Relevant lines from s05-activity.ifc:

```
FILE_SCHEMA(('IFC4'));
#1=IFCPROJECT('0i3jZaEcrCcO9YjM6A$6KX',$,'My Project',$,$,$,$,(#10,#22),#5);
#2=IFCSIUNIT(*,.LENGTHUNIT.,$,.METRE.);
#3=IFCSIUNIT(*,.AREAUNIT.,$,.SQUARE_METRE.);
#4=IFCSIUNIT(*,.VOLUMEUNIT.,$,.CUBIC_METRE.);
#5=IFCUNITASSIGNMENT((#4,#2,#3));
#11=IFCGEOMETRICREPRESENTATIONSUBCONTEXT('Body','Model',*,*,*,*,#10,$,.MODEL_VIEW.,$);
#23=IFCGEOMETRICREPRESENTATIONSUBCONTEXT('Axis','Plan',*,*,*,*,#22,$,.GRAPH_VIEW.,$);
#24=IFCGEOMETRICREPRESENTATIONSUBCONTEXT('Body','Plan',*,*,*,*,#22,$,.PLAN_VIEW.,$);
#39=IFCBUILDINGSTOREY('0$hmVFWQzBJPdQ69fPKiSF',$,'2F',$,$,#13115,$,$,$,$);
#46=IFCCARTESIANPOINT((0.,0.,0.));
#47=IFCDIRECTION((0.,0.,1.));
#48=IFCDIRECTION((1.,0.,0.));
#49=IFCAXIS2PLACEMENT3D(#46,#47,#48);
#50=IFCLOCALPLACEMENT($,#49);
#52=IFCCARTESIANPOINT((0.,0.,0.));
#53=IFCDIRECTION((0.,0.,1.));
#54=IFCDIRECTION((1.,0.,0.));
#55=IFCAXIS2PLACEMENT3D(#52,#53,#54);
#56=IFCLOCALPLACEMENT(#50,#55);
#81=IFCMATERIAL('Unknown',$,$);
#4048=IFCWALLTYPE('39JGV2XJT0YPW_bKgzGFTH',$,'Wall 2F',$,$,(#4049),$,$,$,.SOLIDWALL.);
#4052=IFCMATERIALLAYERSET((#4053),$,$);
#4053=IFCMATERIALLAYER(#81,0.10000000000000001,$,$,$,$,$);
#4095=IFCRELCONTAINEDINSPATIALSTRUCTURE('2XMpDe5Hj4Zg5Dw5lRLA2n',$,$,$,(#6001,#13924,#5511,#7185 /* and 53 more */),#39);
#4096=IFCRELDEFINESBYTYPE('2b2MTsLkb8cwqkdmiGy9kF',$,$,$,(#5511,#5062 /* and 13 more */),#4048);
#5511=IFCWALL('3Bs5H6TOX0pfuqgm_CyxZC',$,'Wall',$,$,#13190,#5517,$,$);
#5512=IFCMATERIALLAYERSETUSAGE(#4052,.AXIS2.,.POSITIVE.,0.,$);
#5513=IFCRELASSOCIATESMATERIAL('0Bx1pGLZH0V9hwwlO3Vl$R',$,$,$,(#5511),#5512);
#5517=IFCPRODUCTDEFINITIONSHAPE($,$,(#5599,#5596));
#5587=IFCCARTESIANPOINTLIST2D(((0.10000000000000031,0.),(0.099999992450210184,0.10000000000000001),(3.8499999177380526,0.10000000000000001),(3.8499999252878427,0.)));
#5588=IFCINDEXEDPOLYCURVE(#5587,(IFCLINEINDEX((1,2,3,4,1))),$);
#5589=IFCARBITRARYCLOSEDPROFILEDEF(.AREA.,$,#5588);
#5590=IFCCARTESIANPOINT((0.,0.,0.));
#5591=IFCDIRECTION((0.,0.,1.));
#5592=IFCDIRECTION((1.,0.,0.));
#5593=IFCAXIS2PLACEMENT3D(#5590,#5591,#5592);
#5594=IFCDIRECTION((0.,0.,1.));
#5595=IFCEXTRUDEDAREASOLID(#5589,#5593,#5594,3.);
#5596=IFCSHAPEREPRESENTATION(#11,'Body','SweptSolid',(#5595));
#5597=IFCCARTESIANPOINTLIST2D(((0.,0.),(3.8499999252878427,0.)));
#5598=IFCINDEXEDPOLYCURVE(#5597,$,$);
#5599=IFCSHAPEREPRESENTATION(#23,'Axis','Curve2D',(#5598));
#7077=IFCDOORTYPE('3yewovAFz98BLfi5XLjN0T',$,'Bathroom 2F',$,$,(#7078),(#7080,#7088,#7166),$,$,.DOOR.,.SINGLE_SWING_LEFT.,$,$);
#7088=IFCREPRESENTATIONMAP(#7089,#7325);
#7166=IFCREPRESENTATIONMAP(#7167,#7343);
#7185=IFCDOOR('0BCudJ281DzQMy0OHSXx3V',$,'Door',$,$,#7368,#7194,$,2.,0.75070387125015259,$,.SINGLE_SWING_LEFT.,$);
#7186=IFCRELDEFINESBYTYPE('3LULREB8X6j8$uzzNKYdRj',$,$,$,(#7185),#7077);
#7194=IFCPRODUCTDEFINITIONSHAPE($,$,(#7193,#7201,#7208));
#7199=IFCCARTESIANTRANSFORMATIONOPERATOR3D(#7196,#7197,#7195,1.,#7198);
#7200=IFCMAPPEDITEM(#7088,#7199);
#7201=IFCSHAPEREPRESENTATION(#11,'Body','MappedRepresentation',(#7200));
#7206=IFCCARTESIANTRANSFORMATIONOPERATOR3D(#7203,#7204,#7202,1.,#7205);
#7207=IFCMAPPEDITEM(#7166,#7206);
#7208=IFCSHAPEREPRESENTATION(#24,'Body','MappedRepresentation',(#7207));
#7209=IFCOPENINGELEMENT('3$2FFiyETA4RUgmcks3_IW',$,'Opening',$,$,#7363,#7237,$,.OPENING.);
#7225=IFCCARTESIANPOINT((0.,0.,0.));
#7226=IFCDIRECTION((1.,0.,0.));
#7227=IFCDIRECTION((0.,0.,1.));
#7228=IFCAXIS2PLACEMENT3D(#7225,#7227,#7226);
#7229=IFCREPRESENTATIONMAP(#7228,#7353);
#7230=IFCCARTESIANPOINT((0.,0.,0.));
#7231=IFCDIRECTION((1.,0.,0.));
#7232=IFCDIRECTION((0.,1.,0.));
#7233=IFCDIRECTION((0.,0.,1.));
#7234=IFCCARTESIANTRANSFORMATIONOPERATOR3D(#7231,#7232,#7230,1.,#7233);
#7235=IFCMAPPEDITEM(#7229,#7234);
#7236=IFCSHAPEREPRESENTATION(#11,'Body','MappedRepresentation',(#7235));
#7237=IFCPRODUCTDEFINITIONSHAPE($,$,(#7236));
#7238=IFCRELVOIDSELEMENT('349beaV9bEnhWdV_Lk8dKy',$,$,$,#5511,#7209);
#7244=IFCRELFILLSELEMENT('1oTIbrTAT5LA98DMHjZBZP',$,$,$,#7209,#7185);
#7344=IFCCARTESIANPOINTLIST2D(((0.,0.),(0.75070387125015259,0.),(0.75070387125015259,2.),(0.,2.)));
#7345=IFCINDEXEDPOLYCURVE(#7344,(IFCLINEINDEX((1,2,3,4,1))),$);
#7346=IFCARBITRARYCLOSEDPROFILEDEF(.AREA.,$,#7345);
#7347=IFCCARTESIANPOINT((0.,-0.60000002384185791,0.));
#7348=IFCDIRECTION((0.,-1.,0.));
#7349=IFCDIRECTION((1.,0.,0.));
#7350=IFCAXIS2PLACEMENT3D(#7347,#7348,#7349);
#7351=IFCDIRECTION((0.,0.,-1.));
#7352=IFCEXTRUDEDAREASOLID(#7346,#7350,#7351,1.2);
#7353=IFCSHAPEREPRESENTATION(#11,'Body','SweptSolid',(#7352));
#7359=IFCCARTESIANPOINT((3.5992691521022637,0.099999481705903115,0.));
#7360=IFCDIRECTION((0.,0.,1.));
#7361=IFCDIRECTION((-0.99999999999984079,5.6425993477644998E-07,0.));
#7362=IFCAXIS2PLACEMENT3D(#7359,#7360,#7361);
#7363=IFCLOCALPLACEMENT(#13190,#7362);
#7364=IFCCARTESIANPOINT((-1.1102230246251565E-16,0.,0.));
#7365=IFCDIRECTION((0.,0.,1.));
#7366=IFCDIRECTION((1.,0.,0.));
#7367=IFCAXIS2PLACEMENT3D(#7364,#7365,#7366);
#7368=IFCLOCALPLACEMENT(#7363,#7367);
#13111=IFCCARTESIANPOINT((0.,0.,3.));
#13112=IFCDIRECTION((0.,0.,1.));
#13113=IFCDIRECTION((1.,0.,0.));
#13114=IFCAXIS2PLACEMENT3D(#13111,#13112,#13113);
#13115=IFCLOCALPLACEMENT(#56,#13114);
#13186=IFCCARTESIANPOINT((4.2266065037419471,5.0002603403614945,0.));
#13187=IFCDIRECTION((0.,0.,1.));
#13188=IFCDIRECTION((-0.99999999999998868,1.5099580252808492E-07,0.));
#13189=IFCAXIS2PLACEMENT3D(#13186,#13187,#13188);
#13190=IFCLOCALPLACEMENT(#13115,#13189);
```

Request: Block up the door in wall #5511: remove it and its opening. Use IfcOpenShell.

```python
import ifcopenshell
import ifcopenshell.api.feature
import ifcopenshell.api.root
import ifcopenshell.geom
import ifcopenshell.util.shape

model = ifcopenshell.open("s05-activity.ifc")
settings = ifcopenshell.geom.settings()


def volume(element):
    """Net volume in cubic metres, openings subtracted."""
    shape = ifcopenshell.geom.create_shape(settings, element)
    return ifcopenshell.util.shape.get_volume(shape.geometry)


door = model.by_guid("0BCudJ281DzQMy0OHSXx3V")
opening = door.FillsVoids[0].RelatingOpeningElement
wall = opening.VoidsElements[0].RelatingBuildingElement
before = volume(wall)

ifcopenshell.api.root.remove_product(model, product=door)
ifcopenshell.api.feature.remove_feature(model, feature=opening)

after = volume(wall)

print(f"wall volume {before:.3f} -> {after:.3f} m3")

model.write("s05-activity_edited.ifc")
```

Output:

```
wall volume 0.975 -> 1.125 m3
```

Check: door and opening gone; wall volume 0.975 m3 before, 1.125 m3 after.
